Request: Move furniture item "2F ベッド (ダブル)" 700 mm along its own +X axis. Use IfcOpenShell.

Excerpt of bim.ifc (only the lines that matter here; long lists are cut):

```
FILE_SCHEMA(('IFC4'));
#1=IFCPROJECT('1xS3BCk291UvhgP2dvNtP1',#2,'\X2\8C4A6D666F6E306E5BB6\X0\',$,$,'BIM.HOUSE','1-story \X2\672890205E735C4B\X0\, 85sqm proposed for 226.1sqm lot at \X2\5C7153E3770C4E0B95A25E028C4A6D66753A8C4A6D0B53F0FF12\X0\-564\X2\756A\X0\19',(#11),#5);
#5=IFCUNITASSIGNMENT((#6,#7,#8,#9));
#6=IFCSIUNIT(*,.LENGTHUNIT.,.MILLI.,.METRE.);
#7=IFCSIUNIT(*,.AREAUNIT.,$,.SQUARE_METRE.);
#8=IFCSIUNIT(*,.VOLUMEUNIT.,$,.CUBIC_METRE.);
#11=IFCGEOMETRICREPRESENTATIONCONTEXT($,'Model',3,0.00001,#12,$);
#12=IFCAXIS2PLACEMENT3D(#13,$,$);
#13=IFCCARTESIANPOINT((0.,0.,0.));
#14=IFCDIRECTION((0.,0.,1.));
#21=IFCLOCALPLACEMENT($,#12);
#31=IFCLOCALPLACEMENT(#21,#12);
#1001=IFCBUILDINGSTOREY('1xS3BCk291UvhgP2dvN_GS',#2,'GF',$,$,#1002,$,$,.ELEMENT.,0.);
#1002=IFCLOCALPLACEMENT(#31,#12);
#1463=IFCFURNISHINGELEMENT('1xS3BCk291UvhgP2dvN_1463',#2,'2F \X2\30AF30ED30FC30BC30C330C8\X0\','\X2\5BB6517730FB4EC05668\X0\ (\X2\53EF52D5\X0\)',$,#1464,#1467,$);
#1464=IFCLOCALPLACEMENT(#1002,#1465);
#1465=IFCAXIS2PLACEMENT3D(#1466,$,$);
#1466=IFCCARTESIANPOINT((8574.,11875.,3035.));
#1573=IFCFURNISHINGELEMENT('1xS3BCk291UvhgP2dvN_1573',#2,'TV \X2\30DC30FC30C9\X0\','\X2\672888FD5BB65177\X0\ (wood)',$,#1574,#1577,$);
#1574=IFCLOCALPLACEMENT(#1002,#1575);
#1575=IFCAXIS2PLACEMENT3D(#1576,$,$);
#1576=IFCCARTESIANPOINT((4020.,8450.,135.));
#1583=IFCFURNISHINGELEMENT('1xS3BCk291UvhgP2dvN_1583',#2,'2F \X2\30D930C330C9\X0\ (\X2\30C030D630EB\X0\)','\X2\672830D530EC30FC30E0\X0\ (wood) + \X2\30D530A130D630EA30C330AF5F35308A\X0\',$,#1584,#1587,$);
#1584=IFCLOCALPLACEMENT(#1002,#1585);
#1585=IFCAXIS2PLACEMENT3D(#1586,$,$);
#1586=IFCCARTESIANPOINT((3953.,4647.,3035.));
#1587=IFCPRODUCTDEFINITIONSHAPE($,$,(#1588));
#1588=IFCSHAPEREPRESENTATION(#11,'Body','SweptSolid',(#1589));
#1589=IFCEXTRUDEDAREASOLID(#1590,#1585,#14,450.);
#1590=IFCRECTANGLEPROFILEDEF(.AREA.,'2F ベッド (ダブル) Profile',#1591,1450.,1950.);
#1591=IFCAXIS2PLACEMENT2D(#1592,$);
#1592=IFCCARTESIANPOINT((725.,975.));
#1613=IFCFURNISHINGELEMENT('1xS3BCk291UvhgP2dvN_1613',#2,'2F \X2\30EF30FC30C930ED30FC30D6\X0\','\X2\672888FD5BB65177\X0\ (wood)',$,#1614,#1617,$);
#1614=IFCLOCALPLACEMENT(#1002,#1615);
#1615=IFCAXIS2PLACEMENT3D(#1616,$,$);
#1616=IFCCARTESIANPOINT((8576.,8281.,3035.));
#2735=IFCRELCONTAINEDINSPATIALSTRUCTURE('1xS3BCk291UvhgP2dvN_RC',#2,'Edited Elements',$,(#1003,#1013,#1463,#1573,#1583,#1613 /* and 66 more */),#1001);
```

```python
import ifcopenshell
import ifcopenshell.api.geometry
import ifcopenshell.util.placement
import ifcopenshell.util.unit

model = ifcopenshell.open("bim.ifc")
unit_scale = ifcopenshell.util.unit.calculate_unit_scale(model)

item = model.by_guid("1xS3BCk291UvhgP2dvN_1583")
matrix = ifcopenshell.util.placement.get_local_placement(item.ObjectPlacement)
matrix[:3, 3] += matrix[:3, 0] * 0.7 / unit_scale
ifcopenshell.api.geometry.edit_object_placement(model, product=item, matrix=matrix, is_si=False)

print(ifcopenshell.util.placement.get_local_placement(item.ObjectPlacement).round(3) + 0.0)

model.write("bim_edited.ifc")
```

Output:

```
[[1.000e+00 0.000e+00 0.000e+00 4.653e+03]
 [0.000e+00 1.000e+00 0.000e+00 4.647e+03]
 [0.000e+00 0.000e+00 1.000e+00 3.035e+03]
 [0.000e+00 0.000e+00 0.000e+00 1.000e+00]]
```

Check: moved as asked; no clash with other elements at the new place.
